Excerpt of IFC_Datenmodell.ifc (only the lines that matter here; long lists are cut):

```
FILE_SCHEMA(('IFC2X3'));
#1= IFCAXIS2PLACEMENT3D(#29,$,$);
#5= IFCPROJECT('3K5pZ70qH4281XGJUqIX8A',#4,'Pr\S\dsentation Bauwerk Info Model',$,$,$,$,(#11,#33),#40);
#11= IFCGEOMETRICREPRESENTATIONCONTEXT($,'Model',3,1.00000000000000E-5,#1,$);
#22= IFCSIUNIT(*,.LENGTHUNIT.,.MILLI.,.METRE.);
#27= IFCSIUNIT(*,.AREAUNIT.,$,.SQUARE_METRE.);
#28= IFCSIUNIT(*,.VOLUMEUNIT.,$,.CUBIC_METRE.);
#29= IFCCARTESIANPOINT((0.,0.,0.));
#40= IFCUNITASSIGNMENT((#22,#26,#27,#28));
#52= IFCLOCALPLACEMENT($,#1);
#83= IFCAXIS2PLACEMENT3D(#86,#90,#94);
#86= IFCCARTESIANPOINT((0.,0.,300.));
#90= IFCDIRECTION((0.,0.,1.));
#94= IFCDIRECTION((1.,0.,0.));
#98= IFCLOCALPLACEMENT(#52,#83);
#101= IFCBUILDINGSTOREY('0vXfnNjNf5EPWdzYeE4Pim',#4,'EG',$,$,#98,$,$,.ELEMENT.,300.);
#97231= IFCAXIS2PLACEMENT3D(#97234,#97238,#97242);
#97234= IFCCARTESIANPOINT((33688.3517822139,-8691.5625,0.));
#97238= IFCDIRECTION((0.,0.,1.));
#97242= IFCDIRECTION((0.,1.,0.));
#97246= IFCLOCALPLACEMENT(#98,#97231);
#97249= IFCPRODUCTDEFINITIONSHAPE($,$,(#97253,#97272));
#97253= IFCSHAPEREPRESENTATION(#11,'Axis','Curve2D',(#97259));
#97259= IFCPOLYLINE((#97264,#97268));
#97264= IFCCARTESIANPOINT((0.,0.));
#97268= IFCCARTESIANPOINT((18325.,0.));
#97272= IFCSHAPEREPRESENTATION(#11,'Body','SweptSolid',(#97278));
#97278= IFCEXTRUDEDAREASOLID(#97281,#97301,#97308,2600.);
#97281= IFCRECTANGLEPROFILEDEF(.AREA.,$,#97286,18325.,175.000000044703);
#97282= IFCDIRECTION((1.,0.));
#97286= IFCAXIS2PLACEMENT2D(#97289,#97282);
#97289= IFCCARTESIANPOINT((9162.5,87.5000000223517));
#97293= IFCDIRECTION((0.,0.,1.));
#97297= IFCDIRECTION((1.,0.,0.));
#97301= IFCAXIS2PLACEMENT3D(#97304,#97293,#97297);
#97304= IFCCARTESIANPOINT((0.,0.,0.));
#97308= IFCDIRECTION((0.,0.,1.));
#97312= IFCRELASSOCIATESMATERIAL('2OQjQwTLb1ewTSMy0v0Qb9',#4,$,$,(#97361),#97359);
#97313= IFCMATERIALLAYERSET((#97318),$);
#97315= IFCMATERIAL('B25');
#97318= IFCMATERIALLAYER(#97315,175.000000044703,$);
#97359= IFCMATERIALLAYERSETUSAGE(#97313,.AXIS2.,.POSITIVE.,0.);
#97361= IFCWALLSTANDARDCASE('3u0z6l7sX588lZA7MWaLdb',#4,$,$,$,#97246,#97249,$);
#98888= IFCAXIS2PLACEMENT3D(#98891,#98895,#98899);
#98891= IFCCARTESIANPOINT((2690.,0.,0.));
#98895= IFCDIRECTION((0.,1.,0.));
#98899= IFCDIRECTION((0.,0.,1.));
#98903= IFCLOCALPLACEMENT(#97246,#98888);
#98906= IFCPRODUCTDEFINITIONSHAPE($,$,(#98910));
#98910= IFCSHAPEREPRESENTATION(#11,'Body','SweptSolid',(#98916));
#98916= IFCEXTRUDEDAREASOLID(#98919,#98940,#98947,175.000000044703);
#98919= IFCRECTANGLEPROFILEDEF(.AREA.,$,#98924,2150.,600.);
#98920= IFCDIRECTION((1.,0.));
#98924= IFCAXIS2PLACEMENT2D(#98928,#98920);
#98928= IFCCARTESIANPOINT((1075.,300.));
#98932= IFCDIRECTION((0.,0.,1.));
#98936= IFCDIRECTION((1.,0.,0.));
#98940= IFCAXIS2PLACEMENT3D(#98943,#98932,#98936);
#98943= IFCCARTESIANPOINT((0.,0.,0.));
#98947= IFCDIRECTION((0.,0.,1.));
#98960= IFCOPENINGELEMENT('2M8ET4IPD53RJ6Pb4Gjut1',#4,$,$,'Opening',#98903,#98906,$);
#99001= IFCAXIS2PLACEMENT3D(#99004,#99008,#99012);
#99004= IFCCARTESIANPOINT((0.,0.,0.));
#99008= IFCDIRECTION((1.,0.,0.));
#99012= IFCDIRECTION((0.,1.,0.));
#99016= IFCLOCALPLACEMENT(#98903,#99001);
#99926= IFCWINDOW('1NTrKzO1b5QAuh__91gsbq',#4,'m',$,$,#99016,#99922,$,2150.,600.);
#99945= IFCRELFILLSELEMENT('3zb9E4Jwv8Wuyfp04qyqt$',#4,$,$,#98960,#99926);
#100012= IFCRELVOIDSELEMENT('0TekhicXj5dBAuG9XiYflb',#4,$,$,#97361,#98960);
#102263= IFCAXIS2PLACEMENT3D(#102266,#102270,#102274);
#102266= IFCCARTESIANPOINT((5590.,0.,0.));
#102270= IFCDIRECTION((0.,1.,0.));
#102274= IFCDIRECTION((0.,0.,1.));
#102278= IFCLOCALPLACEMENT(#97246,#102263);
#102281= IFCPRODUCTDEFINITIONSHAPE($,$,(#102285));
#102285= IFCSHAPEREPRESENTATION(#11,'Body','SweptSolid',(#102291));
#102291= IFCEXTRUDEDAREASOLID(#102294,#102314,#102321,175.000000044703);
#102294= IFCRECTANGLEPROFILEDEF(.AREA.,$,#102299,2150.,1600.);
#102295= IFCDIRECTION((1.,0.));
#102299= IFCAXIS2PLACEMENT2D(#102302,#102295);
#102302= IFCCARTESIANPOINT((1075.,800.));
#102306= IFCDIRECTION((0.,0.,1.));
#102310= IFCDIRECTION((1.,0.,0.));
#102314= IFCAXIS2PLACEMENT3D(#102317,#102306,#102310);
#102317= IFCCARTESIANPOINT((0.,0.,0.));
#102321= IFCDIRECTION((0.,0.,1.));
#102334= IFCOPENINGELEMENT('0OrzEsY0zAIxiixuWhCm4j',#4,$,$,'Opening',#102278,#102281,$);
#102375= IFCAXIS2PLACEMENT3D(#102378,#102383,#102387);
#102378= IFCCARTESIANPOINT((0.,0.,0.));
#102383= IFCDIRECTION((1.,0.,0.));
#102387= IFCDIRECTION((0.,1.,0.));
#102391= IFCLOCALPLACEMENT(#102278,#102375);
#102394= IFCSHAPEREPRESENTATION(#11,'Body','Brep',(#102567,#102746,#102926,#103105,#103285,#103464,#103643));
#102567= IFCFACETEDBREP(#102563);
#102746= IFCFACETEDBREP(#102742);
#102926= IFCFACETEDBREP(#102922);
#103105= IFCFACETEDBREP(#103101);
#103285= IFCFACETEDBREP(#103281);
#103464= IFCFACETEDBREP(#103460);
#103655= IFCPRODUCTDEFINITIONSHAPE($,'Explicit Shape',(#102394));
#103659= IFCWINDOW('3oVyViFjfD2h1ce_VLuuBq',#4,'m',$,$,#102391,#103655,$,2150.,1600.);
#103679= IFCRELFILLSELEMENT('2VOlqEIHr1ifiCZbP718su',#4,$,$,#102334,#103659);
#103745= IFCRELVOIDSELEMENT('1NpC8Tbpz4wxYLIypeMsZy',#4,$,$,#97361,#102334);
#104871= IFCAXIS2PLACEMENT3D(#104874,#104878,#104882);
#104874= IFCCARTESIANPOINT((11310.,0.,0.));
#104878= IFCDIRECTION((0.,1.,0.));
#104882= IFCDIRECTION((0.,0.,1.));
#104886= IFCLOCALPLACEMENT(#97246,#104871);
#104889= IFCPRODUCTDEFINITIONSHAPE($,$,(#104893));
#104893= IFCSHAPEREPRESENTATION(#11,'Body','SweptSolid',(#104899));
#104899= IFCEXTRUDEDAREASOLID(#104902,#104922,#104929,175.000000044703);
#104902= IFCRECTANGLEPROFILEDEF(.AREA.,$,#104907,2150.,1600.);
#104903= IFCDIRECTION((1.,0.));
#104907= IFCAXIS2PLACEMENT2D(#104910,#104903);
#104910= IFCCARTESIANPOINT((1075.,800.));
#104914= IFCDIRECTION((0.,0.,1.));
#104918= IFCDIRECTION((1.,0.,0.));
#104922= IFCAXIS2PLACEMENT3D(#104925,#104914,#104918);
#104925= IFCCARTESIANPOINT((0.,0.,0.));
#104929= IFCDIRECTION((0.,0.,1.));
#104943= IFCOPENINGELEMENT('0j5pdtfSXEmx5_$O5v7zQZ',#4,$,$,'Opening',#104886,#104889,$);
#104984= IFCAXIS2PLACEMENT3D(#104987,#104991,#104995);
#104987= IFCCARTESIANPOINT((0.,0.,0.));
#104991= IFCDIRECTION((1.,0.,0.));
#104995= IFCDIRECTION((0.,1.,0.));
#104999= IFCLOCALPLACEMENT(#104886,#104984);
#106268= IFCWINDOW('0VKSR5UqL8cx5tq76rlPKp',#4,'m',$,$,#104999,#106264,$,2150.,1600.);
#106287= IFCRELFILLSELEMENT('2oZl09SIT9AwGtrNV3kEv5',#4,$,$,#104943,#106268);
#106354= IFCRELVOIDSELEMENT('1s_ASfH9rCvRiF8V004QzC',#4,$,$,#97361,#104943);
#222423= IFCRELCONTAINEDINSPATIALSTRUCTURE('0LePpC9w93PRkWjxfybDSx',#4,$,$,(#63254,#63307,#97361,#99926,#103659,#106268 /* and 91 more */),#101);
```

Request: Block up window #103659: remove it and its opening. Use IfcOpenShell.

```python
import ifcopenshell
import ifcopenshell.api.feature
import ifcopenshell.api.root
import ifcopenshell.geom
import ifcopenshell.util.shape

model = ifcopenshell.open("IFC_Datenmodell.ifc")
settings = ifcopenshell.geom.settings()


def volume(element):
    """Net volume in cubic metres, openings subtracted."""
    shape = ifcopenshell.geom.create_shape(settings, element)
    return ifcopenshell.util.shape.get_volume(shape.geometry)


window = model.by_id(103659)
opening = window.FillsVoids[0].RelatingOpeningElement
wall = opening.VoidsElements[0].RelatingBuildingElement
before = volume(wall)

ifcopenshell.api.root.remove_product(model, product=window)
ifcopenshell.api.feature.remove_feature(model, feature=opening)

after = volume(wall)

print(f"wall volume {before:.3f} -> {after:.3f} m3")

model.write("IFC_Datenmodell_v2.ifc")
```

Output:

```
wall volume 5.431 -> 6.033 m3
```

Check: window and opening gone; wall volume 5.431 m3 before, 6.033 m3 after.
